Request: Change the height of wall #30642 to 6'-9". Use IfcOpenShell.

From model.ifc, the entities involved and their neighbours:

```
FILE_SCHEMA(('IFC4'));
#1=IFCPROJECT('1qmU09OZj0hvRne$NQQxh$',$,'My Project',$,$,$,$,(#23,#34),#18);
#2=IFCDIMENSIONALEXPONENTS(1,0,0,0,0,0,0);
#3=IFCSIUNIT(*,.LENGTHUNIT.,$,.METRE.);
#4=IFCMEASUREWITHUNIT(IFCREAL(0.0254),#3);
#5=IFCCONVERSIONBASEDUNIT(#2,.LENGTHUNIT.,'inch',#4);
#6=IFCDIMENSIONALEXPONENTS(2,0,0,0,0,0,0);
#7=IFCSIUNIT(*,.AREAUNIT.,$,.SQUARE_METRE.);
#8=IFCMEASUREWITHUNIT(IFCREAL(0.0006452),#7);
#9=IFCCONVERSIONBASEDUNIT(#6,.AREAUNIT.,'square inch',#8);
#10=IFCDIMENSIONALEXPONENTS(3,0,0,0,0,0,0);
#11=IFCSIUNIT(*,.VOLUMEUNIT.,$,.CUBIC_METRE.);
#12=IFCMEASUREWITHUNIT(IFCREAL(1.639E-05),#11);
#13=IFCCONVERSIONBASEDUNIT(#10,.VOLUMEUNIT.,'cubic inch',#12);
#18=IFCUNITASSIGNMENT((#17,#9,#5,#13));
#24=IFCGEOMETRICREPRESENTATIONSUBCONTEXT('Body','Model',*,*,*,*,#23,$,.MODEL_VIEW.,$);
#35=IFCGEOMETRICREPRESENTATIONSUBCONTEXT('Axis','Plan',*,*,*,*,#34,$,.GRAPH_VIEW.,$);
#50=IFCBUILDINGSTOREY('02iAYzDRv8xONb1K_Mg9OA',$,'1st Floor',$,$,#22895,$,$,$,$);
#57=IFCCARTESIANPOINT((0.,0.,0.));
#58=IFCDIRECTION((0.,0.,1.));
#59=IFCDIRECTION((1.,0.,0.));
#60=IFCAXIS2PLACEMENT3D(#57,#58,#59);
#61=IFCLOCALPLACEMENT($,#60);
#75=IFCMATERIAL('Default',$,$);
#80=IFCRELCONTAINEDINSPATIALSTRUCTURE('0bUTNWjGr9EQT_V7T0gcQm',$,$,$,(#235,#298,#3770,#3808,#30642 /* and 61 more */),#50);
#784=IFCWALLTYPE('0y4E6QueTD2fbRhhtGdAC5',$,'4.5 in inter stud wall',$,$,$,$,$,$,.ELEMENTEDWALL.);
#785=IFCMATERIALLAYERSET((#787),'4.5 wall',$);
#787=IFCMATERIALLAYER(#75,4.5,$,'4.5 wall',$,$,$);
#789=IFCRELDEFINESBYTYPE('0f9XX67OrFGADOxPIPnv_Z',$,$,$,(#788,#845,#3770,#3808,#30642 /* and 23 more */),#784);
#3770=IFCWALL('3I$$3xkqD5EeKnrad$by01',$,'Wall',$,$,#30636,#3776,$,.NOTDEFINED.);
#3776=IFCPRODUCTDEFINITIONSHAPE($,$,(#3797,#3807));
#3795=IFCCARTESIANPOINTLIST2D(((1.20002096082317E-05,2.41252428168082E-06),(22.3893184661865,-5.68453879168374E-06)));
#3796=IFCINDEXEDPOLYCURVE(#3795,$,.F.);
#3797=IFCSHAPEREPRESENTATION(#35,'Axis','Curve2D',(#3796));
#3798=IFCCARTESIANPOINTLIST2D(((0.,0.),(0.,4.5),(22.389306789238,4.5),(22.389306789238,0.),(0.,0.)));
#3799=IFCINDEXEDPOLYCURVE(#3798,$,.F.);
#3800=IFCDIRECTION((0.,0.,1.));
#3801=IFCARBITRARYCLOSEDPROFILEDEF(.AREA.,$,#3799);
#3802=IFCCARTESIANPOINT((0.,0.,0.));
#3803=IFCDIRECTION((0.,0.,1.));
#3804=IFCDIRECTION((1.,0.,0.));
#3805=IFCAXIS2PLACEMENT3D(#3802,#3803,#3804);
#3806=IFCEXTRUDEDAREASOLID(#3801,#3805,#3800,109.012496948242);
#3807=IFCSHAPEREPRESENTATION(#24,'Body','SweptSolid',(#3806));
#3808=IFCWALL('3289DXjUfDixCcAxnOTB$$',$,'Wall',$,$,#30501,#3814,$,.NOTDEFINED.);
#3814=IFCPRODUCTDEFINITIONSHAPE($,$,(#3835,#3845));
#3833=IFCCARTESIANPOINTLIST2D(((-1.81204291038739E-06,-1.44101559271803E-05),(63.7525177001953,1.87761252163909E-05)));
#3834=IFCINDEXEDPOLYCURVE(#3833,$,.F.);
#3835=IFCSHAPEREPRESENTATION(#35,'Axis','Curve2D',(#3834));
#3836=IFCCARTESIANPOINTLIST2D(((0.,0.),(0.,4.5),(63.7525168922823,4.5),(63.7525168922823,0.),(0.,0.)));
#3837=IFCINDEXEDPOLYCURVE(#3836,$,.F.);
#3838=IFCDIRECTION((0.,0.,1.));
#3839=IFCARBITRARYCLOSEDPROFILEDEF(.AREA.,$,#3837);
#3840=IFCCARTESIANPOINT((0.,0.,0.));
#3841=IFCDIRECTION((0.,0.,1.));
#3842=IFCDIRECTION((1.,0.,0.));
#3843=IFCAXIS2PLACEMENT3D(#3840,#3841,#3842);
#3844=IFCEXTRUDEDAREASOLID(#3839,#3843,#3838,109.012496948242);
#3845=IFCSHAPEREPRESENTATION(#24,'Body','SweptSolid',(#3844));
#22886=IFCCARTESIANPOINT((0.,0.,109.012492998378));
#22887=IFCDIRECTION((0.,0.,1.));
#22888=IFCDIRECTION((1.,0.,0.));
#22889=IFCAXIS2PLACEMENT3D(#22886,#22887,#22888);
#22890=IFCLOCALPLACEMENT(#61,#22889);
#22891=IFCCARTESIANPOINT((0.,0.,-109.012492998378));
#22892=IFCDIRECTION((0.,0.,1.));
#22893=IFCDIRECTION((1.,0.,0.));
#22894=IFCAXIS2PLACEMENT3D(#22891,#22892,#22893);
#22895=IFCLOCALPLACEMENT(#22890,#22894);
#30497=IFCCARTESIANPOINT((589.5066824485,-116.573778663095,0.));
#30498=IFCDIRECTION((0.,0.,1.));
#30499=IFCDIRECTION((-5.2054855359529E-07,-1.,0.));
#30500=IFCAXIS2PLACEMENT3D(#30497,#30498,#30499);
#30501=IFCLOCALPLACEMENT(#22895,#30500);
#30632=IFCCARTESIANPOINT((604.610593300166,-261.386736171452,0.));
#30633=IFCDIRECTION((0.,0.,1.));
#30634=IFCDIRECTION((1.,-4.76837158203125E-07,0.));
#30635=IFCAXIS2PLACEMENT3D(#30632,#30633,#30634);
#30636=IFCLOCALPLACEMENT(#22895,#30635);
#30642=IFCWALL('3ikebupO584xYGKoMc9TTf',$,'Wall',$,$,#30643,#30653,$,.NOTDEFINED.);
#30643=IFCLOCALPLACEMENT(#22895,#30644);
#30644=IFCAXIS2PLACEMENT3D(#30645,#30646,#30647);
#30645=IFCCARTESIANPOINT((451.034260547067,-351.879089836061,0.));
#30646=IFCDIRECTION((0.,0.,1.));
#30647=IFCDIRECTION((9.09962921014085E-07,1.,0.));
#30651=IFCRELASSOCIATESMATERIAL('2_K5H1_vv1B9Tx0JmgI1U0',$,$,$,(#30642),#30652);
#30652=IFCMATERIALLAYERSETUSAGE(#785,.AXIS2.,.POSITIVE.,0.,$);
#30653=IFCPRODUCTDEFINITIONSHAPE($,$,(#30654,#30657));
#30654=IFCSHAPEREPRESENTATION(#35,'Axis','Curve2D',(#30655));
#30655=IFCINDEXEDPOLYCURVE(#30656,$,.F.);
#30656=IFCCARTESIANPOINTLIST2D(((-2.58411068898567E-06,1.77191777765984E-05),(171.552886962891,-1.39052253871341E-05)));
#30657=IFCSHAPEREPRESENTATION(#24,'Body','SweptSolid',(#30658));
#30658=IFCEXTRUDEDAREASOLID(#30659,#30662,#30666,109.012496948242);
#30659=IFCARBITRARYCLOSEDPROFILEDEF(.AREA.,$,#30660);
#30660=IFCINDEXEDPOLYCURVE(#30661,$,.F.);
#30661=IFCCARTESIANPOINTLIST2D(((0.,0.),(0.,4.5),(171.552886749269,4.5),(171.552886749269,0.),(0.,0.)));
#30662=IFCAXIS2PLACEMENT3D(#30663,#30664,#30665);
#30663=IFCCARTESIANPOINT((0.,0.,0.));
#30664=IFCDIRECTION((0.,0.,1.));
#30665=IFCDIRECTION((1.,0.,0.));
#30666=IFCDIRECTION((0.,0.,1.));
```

```python
import ifcopenshell
import ifcopenshell.geom
import ifcopenshell.util.representation
import ifcopenshell.util.shape
import ifcopenshell.util.unit

model = ifcopenshell.open("model.ifc")
unit_scale = ifcopenshell.util.unit.calculate_unit_scale(model)
settings = ifcopenshell.geom.settings()


def volume(element):
    """Net volume in cubic metres, openings subtracted."""
    shape = ifcopenshell.geom.create_shape(settings, element)
    return ifcopenshell.util.shape.get_volume(shape.geometry)


wall = model.by_guid("3ikebupO584xYGKoMc9TTf")
before = volume(wall)

body = ifcopenshell.util.representation.get_representation(wall, "Model", "Body")
solid = body.Items[0]
old_height = solid.Depth
solid.Depth = 81 * 0.0254 / unit_scale
after = volume(wall)

print(f"height {old_height:g} -> {solid.Depth:g}, volume {before:.3f} -> {after:.3f} m3")

model.write("model_v2.ifc")
```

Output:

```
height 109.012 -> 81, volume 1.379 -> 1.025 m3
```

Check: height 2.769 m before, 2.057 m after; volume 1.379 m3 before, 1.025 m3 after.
